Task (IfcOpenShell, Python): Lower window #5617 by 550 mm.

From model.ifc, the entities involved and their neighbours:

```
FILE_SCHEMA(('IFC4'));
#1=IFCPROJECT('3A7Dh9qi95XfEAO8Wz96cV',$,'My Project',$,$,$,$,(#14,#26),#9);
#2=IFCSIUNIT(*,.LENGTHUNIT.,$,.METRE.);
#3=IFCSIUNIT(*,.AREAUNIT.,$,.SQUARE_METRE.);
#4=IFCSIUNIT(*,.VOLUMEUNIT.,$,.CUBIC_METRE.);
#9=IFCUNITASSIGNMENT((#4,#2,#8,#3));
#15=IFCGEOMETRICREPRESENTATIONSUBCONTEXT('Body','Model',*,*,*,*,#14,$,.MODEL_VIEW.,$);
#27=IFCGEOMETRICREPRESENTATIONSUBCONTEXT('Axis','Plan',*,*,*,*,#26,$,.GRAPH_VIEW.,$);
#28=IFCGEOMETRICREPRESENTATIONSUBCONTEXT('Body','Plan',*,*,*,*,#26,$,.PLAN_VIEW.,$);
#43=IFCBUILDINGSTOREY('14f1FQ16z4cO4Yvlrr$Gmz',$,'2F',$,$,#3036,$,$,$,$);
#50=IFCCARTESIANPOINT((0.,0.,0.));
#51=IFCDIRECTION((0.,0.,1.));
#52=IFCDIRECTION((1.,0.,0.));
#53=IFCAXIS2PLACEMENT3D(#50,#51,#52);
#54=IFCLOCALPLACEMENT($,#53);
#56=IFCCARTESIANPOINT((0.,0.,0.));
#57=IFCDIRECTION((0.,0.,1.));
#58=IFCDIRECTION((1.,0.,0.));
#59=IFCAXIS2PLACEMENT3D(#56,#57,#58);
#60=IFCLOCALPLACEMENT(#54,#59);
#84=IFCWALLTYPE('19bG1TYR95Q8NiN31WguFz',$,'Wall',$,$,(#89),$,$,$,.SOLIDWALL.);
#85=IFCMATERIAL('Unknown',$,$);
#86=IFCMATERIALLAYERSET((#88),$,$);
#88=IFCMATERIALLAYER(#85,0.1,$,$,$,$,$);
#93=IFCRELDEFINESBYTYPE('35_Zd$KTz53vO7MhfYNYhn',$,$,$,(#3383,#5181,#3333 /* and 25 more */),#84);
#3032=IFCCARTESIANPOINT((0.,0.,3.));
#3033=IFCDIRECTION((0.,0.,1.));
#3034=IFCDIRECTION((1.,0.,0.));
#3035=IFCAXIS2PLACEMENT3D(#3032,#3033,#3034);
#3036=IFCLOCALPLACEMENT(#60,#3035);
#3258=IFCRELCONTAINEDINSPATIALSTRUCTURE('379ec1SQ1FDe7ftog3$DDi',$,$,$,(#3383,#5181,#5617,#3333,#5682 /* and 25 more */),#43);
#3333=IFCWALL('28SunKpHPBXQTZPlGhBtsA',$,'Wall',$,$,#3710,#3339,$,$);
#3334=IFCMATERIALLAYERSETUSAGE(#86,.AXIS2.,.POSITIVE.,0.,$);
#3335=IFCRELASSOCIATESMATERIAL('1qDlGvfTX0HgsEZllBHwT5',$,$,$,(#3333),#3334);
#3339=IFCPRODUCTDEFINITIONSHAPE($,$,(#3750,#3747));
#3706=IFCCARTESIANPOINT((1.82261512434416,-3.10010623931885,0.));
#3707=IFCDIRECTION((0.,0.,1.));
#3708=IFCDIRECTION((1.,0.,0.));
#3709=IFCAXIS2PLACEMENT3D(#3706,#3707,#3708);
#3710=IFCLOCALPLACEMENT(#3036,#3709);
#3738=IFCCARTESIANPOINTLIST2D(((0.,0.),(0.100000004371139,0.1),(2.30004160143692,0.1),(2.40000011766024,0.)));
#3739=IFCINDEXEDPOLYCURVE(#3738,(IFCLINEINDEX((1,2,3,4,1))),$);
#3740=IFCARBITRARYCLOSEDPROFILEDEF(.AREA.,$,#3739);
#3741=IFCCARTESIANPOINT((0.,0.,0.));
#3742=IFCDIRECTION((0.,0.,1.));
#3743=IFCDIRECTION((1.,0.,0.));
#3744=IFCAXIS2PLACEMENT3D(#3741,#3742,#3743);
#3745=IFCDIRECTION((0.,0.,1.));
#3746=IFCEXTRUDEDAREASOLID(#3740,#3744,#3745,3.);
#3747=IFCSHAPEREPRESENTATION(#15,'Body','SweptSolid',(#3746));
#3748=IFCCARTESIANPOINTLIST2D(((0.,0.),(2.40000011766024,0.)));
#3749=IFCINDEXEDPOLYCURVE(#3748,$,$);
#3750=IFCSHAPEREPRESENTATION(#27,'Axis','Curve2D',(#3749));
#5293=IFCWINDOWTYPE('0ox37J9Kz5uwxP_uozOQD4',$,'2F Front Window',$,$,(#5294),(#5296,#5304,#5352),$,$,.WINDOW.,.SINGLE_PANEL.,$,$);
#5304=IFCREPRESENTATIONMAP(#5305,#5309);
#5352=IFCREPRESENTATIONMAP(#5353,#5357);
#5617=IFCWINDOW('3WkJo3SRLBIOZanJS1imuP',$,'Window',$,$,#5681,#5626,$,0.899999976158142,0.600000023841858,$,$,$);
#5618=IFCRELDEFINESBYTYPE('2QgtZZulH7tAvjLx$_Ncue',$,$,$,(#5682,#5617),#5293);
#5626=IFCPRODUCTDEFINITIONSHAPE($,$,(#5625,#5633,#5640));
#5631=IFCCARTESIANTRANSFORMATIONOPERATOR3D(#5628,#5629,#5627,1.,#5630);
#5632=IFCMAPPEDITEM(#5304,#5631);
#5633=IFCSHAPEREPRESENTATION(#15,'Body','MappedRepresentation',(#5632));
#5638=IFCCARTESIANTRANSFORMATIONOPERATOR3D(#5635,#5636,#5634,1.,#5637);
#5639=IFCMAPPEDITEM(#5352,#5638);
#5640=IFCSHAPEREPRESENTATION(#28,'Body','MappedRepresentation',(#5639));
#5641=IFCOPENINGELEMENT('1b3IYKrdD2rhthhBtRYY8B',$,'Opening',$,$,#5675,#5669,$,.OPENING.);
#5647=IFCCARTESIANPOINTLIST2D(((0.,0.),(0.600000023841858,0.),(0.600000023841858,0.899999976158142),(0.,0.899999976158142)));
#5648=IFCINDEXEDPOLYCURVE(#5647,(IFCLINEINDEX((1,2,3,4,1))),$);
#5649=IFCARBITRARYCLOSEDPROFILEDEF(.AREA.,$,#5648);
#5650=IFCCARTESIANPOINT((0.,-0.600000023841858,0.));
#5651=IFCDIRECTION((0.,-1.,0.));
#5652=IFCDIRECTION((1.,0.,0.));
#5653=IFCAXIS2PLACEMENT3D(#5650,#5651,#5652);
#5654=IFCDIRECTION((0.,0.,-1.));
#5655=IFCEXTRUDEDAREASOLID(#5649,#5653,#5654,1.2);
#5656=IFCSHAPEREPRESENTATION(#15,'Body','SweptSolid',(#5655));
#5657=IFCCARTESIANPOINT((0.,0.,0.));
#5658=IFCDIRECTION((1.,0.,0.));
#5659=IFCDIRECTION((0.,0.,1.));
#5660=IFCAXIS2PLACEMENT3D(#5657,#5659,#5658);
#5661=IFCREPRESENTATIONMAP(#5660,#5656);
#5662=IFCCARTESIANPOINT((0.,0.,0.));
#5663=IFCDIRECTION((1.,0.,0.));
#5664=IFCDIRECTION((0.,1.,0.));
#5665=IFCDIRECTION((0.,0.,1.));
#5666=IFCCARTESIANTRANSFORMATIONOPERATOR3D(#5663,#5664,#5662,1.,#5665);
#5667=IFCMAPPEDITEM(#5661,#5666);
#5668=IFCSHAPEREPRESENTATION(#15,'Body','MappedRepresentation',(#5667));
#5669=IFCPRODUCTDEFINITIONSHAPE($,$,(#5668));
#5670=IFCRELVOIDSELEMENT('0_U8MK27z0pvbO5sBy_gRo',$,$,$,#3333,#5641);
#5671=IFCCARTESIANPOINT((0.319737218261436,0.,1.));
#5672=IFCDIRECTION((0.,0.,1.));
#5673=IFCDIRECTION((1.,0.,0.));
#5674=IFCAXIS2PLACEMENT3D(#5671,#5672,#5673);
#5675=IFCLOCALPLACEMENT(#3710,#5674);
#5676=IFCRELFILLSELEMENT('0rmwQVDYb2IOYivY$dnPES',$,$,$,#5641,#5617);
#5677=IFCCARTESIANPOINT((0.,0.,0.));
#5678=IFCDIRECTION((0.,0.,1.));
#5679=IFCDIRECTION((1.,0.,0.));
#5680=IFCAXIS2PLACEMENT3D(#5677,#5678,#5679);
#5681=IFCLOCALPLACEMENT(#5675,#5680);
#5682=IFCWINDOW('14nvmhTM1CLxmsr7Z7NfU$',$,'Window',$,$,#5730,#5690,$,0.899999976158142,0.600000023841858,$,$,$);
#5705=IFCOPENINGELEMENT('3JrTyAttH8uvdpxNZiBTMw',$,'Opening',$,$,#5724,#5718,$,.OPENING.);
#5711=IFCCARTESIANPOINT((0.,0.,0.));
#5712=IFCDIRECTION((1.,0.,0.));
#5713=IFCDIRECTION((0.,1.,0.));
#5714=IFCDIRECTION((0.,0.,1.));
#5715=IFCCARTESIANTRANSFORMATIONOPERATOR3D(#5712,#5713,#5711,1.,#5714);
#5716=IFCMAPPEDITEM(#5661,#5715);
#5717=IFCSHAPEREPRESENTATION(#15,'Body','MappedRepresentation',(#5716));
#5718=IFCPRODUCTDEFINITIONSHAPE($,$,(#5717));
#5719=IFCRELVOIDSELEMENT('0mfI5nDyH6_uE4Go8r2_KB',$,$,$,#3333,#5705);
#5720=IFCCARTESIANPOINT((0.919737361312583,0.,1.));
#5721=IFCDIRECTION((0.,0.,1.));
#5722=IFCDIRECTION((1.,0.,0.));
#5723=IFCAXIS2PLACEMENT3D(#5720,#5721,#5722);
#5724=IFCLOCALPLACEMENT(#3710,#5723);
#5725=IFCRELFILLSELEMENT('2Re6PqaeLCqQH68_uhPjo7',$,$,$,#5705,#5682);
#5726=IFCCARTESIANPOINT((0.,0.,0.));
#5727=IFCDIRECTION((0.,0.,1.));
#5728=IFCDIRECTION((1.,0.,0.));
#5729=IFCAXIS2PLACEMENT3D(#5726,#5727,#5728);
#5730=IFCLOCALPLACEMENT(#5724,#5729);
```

```python
import numpy as np
import ifcopenshell
import ifcopenshell.api.geometry
import ifcopenshell.util.placement
import ifcopenshell.util.unit

model = ifcopenshell.open("model.ifc")
unit_scale = ifcopenshell.util.unit.calculate_unit_scale(model)

window = model.by_guid("3WkJo3SRLBIOZanJS1imuP")
opening = window.FillsVoids[0].RelatingOpeningElement
dz = -0.55 / unit_scale

shift = np.array([0.0, 0.0, dz])
# The window is placed relative to its opening, so it follows when the opening moves.
matrix = ifcopenshell.util.placement.get_local_placement(opening.ObjectPlacement)
matrix[:3, 3] += shift
ifcopenshell.api.geometry.edit_object_placement(
    model, product=opening, matrix=matrix, is_si=False, should_transform_children=True
)

print(f"moved by {dz * unit_scale:+.3f} m")

model.write("model_edited.ifc")
```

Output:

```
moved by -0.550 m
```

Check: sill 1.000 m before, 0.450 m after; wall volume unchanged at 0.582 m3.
